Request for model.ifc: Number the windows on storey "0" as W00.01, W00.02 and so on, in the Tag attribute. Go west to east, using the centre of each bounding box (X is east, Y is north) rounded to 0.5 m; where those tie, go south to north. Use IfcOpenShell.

First a look at what the model holds.

```python
import ifcopenshell
import ifcopenshell.util.element
import ifcopenshell.util.placement

model = ifcopenshell.open("model.ifc")
print(model.schema)
storey = next(s for s in model.by_type("IfcBuildingStorey") if s.Name == "0")
windows = [e for e in ifcopenshell.util.element.get_decomposition(storey) if e.is_a("IfcWindow")]
for e in sorted(windows, key=lambda e: e.id()):
    origin = ifcopenshell.util.placement.get_local_placement(e.ObjectPlacement)[:3, 3]
    print(e.id(), e.Tag, e.Name, origin.round(2) + 0.0, sep=" | ")
```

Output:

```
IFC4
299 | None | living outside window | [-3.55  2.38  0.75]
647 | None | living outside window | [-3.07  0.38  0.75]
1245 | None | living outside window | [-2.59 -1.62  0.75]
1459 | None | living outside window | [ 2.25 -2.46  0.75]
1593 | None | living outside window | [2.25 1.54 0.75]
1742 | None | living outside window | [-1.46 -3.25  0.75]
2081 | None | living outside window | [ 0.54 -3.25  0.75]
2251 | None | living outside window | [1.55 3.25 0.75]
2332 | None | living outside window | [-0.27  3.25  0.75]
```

```python
import ifcopenshell
import ifcopenshell.geom
import ifcopenshell.util.element
import ifcopenshell.util.shape

model = ifcopenshell.open("model.ifc")
settings = ifcopenshell.geom.settings()
settings.set("use-world-coords", True)


def centre(element):
    shape = ifcopenshell.geom.create_shape(settings, element)
    return ifcopenshell.util.shape.get_bbox_centroid(shape.geometry)


storey = next(s for s in model.by_type("IfcBuildingStorey") if s.Name == "0")
windows = [e for e in ifcopenshell.util.element.get_decomposition(storey) if e.is_a("IfcWindow")]

# Insertion points can sit at a corner or the storey origin, so sort by the geometry (in metres).
centres = {e: centre(e) for e in windows}
windows.sort(key=lambda e: (round(centres[e][0] / 0.5), centres[e][1]))

for i, e in enumerate(windows, start=1):
    number = f"W00.{i:02d}"
    e.Tag = number
    print(e.id(), number)

model.write("model-out.ifc")
```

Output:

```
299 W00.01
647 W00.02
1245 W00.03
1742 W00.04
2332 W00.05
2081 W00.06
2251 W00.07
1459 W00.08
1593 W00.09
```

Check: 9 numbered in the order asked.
